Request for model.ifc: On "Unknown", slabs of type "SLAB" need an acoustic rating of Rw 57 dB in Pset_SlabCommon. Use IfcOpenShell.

First a look at what the model holds.

```python
import ifcopenshell
import ifcopenshell.util.element

model = ifcopenshell.open("model.ifc")
print(model.schema)
storey = next(s for s in model.by_type("IfcBuildingStorey") if s.Name == "Unknown")
slabs = [e for e in ifcopenshell.util.element.get_decomposition(storey) if e.is_a("IfcSlab")]
seen = {}
for e in slabs:
    element_type = ifcopenshell.util.element.get_type(e)
    key = (element_type.Name if element_type != e and element_type else None, ifcopenshell.util.element.get_pset(e, "Pset_SlabCommon", "AcousticRating"))
    seen[key] = seen.get(key, 0) + 1
for (name, value), count in sorted(seen.items(), key=str):
    print(count, "x", name, "|", value)
```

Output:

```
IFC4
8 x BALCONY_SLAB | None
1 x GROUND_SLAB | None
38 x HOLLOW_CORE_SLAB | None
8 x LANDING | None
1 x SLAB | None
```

```python
import ifcopenshell
import ifcopenshell.api.pset
import ifcopenshell.util.element

model = ifcopenshell.open("model.ifc")

storey = next(s for s in model.by_type("IfcBuildingStorey") if s.Name == "Unknown")
slabs = [e for e in ifcopenshell.util.element.get_decomposition(storey) if e.is_a("IfcSlab")]

count = 0
for e in slabs:
    element_type = ifcopenshell.util.element.get_type(e)
    if element_type in (None, e) or element_type.Name != "SLAB":
        continue
    found = ifcopenshell.util.element.get_pset(e, "Pset_SlabCommon", should_inherit=False)
    if found:
        pset = model.by_id(found["id"])
        if len(ifcopenshell.util.element.get_elements_by_pset(pset)) > 1:
            pset = ifcopenshell.api.pset.unshare_pset(model, products=[e], pset=pset)[0]
    else:
        pset = ifcopenshell.api.pset.add_pset(model, product=e, name="Pset_SlabCommon")
    ifcopenshell.api.pset.edit_pset(model, pset=pset, properties={"AcousticRating": "Rw 57 dB"})
    count += 1

print(count, "slabs updated")

model.write("model_v2.ifc")
```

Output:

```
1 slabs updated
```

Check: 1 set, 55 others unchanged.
